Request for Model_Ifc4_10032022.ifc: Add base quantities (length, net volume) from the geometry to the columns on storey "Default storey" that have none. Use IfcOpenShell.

First a look at what the model holds.

```python
import ifcopenshell
import ifcopenshell.util.element
import ifcopenshell.util.unit

model = ifcopenshell.open("Model_Ifc4_10032022.ifc")
print(model.schema)
for unit_type in ("LENGTHUNIT", "AREAUNIT", "VOLUMEUNIT"):
    print(unit_type, ifcopenshell.util.unit.calculate_unit_scale(model, unit_type))
storey = next(s for s in model.by_type("IfcBuildingStorey") if s.Name == "Default storey")
columns = [e for e in ifcopenshell.util.element.get_decomposition(storey) if e.is_a("IfcColumn")]
for e in sorted(columns, key=lambda e: e.id()):
    print(e.id(), e.is_a(), e.Name, list(ifcopenshell.util.element.get_psets(e, qtos_only=True)), sep=" | ")
```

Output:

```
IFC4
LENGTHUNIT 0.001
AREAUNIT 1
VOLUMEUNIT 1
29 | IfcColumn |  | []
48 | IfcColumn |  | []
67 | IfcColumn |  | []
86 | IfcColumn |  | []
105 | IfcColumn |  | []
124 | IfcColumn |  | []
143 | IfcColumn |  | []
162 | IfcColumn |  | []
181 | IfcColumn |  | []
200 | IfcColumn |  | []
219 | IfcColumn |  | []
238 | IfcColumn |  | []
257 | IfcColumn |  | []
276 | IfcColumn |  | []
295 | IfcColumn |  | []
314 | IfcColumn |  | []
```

```python
import ifcopenshell
import ifcopenshell.api.pset
import ifcopenshell.geom
import ifcopenshell.util.element
import ifcopenshell.util.shape
import ifcopenshell.util.unit

model = ifcopenshell.open("Model_Ifc4_10032022.ifc")
unit_scale = ifcopenshell.util.unit.calculate_unit_scale(model)
volume_scale = ifcopenshell.util.unit.calculate_unit_scale(model, "VOLUMEUNIT")
settings = ifcopenshell.geom.settings()

storey = next(s for s in model.by_type("IfcBuildingStorey") if s.Name == "Default storey")
columns = [e for e in ifcopenshell.util.element.get_decomposition(storey) if e.is_a("IfcColumn")]

for e in sorted(columns, key=lambda e: e.id()):
    if ifcopenshell.util.element.get_psets(e, qtos_only=True, should_inherit=False):
        continue
    # Geometry comes back in metres, in the element's own axes.
    shape = ifcopenshell.geom.create_shape(settings, e)
    values = {
        "Length": ifcopenshell.util.shape.get_z(shape.geometry) / unit_scale,
        "NetVolume": ifcopenshell.util.shape.get_volume(shape.geometry) / volume_scale,
    }
    qto = ifcopenshell.api.pset.add_qto(model, product=e, name="Qto_ColumnBaseQuantities")
    ifcopenshell.api.pset.edit_qto(model, qto=qto, properties=values)
    print(e.id(), {k: round(v, 3) for k, v in values.items()})

model.write("Model_Ifc4_10032022_v2.ifc")
```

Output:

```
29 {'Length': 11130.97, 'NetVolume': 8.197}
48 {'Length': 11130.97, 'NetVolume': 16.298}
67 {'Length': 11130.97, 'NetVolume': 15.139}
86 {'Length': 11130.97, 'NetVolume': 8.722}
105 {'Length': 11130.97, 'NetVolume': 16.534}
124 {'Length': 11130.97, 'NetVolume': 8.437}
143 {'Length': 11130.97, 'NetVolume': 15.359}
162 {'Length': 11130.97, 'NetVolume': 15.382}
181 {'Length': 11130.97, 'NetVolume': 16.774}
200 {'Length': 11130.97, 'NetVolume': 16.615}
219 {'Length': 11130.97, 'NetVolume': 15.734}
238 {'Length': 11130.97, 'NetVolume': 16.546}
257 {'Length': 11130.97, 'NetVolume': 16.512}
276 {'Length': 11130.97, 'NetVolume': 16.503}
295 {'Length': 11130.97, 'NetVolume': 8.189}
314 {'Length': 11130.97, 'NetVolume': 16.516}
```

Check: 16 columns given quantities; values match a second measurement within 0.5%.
